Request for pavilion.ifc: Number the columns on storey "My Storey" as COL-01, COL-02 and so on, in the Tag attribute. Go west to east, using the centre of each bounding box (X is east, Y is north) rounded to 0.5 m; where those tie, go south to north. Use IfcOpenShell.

First a look at what the model holds.

```python
import ifcopenshell
import ifcopenshell.util.element
import ifcopenshell.util.placement

model = ifcopenshell.open("pavilion.ifc")
print(model.schema)
storey = next(s for s in model.by_type("IfcBuildingStorey") if s.Name == "My Storey")
columns = [e for e in ifcopenshell.util.element.get_decomposition(storey) if e.is_a("IfcColumn")]
for e in sorted(columns, key=lambda e: e.id()):
    origin = ifcopenshell.util.placement.get_local_placement(e.ObjectPlacement)[:3, 3]
    print(e.id(), e.Tag, e.Name, origin.round(2) + 0.0, sep=" | ")
```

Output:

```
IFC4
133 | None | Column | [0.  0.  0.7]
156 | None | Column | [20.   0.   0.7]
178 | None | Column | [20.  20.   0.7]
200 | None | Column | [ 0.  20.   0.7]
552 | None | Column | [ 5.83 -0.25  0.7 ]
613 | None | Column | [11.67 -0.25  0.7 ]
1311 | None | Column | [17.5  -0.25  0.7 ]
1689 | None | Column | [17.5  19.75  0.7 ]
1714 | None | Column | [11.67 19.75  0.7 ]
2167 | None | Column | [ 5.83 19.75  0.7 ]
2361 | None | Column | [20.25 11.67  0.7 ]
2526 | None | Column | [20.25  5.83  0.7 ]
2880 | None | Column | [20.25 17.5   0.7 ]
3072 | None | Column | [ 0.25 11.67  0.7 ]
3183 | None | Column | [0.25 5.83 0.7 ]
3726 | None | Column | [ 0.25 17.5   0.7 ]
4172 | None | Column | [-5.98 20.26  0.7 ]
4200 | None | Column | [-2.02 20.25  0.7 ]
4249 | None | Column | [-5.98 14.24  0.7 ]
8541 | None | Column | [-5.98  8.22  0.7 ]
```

```python
import ifcopenshell
import ifcopenshell.geom
import ifcopenshell.util.element
import ifcopenshell.util.shape

model = ifcopenshell.open("pavilion.ifc")
settings = ifcopenshell.geom.settings()
settings.set("use-world-coords", True)


def centre(element):
    shape = ifcopenshell.geom.create_shape(settings, element)
    return ifcopenshell.util.shape.get_bbox_centroid(shape.geometry)


storey = next(s for s in model.by_type("IfcBuildingStorey") if s.Name == "My Storey")
columns = [e for e in ifcopenshell.util.element.get_decomposition(storey) if e.is_a("IfcColumn")]

# Insertion points can sit at a corner or the storey origin, so sort by the geometry (in metres).
centres = {e: centre(e) for e in columns}
columns.sort(key=lambda e: (round(centres[e][0] / 0.5), centres[e][1]))

for i, e in enumerate(columns, start=1):
    number = f"COL-{i:02d}"
    e.Tag = number
    print(e.id(), number)

model.write("pavilion_edited.ifc")
```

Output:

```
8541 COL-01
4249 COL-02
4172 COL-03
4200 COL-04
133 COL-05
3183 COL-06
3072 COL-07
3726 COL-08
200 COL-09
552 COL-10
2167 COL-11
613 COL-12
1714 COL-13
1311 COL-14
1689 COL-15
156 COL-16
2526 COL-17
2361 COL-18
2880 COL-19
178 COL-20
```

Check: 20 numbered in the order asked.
